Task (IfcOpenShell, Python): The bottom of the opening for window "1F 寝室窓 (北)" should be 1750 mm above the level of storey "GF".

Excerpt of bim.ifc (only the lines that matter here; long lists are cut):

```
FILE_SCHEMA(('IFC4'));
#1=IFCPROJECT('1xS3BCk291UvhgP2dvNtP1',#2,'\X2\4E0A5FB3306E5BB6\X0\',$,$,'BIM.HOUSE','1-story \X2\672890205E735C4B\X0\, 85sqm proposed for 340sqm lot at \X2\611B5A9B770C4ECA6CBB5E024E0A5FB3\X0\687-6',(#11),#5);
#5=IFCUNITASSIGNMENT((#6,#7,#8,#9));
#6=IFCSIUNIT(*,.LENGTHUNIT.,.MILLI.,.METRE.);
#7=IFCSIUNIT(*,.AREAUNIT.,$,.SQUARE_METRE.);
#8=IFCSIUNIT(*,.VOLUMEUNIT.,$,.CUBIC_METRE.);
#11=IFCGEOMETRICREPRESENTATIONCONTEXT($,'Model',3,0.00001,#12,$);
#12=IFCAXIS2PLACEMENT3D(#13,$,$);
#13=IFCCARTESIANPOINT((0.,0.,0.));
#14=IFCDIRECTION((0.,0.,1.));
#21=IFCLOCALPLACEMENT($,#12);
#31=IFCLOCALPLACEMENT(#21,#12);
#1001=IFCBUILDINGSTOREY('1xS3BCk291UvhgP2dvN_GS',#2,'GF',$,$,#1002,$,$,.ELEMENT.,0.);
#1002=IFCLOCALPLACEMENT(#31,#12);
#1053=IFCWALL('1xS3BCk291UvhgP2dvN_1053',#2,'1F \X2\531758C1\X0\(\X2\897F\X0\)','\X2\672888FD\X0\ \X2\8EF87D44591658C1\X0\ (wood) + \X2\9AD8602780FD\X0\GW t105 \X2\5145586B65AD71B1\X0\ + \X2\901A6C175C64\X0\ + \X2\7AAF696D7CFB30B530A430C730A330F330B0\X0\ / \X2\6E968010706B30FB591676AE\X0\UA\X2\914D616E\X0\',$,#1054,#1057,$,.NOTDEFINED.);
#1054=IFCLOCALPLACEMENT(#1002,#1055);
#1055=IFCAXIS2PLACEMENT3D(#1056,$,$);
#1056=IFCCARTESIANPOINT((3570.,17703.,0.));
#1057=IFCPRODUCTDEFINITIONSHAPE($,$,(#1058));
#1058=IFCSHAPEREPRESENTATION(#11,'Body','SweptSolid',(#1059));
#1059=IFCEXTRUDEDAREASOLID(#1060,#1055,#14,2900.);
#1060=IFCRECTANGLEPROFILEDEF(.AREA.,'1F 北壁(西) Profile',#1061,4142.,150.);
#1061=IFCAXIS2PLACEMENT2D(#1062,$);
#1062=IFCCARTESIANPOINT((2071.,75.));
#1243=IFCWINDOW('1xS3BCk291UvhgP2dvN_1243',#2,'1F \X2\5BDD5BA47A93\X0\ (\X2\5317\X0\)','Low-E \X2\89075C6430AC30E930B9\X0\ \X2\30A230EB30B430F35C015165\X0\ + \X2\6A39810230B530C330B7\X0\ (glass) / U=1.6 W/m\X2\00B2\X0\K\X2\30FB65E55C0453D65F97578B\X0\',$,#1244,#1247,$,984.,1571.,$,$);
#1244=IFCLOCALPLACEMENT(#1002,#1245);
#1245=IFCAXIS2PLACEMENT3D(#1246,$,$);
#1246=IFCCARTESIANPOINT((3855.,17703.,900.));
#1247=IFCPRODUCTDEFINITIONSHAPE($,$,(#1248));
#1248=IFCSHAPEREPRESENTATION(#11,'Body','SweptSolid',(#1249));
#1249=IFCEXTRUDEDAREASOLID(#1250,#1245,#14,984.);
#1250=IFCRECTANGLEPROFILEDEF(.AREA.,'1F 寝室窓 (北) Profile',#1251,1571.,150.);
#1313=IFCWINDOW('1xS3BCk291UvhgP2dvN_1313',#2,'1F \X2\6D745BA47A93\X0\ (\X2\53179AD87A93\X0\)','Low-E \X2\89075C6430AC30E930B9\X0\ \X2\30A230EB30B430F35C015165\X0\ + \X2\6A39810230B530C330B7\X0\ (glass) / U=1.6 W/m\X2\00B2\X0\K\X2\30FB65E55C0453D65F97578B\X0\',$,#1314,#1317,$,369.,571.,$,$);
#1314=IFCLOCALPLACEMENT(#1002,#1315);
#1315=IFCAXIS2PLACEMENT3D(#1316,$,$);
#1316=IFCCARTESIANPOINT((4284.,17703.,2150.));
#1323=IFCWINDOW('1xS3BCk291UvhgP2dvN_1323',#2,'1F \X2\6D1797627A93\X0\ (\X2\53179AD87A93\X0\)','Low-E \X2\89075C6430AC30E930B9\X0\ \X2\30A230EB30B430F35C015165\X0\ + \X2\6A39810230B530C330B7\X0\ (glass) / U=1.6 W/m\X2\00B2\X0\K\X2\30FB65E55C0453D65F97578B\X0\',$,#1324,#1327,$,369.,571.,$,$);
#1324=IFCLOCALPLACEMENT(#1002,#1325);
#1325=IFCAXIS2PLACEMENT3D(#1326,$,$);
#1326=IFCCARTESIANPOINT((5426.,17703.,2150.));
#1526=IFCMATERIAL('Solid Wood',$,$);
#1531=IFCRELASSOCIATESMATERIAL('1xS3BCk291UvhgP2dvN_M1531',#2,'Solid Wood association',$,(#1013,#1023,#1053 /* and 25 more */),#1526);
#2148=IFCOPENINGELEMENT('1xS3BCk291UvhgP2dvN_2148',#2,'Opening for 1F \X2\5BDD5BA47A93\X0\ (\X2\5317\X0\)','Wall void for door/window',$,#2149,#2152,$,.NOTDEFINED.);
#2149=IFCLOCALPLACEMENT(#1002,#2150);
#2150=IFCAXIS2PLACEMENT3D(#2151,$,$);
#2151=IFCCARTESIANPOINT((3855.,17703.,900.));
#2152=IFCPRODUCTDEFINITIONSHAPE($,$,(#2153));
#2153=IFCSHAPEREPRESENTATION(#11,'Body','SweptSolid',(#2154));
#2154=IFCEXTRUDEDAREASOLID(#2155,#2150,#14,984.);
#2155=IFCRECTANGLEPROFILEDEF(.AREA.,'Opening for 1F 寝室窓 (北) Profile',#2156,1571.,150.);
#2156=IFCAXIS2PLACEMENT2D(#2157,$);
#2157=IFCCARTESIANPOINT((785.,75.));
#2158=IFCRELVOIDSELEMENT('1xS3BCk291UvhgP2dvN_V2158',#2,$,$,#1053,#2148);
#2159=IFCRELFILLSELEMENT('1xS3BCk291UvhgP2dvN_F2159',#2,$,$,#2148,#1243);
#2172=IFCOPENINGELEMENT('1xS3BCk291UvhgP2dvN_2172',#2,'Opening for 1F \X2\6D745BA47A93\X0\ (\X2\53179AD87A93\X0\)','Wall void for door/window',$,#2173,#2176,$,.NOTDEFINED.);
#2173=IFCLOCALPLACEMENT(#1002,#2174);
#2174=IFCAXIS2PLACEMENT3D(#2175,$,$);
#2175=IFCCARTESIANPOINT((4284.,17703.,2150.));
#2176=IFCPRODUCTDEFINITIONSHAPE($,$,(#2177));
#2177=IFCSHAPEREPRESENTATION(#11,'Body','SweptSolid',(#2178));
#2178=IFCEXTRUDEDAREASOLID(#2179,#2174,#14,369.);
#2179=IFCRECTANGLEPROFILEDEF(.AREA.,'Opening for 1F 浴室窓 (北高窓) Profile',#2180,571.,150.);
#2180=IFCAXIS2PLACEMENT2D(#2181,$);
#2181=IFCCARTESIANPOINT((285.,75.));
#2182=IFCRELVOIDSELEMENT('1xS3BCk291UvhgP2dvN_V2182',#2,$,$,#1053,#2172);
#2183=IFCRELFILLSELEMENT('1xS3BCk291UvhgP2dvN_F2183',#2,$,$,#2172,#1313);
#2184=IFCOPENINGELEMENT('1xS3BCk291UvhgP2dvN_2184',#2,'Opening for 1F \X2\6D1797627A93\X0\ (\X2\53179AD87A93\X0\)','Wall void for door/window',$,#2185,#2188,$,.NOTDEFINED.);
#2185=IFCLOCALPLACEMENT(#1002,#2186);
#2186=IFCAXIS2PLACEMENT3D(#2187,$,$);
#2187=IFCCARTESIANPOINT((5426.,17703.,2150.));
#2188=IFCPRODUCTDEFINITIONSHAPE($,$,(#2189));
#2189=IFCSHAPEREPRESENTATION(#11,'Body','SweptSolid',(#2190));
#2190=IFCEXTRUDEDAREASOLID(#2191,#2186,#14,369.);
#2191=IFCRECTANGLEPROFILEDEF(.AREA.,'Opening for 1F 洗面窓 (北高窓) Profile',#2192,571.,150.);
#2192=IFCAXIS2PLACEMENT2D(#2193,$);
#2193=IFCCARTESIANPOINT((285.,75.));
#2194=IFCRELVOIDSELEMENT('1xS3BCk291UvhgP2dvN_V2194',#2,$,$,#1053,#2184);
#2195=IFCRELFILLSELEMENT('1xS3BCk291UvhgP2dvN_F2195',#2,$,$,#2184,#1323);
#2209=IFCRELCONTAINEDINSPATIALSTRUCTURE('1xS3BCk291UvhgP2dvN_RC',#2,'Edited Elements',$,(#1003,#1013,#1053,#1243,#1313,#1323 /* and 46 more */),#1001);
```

```python
import numpy as np
import ifcopenshell
import ifcopenshell.api.geometry
import ifcopenshell.geom
import ifcopenshell.util.element
import ifcopenshell.util.placement
import ifcopenshell.util.shape
import ifcopenshell.util.unit

model = ifcopenshell.open("bim.ifc")
unit_scale = ifcopenshell.util.unit.calculate_unit_scale(model)

window = model.by_guid("1xS3BCk291UvhgP2dvN_1243")
opening = window.FillsVoids[0].RelatingOpeningElement
storey = ifcopenshell.util.element.get_container(window, ifc_class="IfcBuildingStorey")
level = ifcopenshell.util.placement.get_local_placement(storey.ObjectPlacement)[2, 3]

# The opening's origin need not be at the sill, so measure its lowest point.
shape = ifcopenshell.geom.create_shape(ifcopenshell.geom.settings(), opening)
bottom = ifcopenshell.util.shape.get_shape_bottom_elevation(shape, shape.geometry) / unit_scale
dz = level + 1.75 / unit_scale - bottom

shift = np.array([0.0, 0.0, dz])
# The window is not placed relative to its opening, so move both.
for product in (opening, window):
    matrix = ifcopenshell.util.placement.get_local_placement(product.ObjectPlacement)
    matrix[:3, 3] += shift
    ifcopenshell.api.geometry.edit_object_placement(model, product=product, matrix=matrix, is_si=False)

print(f"moved by {dz * unit_scale:+.3f} m")

model.write("bim-out.ifc")
```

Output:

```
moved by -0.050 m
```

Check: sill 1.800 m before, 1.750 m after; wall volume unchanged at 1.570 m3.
